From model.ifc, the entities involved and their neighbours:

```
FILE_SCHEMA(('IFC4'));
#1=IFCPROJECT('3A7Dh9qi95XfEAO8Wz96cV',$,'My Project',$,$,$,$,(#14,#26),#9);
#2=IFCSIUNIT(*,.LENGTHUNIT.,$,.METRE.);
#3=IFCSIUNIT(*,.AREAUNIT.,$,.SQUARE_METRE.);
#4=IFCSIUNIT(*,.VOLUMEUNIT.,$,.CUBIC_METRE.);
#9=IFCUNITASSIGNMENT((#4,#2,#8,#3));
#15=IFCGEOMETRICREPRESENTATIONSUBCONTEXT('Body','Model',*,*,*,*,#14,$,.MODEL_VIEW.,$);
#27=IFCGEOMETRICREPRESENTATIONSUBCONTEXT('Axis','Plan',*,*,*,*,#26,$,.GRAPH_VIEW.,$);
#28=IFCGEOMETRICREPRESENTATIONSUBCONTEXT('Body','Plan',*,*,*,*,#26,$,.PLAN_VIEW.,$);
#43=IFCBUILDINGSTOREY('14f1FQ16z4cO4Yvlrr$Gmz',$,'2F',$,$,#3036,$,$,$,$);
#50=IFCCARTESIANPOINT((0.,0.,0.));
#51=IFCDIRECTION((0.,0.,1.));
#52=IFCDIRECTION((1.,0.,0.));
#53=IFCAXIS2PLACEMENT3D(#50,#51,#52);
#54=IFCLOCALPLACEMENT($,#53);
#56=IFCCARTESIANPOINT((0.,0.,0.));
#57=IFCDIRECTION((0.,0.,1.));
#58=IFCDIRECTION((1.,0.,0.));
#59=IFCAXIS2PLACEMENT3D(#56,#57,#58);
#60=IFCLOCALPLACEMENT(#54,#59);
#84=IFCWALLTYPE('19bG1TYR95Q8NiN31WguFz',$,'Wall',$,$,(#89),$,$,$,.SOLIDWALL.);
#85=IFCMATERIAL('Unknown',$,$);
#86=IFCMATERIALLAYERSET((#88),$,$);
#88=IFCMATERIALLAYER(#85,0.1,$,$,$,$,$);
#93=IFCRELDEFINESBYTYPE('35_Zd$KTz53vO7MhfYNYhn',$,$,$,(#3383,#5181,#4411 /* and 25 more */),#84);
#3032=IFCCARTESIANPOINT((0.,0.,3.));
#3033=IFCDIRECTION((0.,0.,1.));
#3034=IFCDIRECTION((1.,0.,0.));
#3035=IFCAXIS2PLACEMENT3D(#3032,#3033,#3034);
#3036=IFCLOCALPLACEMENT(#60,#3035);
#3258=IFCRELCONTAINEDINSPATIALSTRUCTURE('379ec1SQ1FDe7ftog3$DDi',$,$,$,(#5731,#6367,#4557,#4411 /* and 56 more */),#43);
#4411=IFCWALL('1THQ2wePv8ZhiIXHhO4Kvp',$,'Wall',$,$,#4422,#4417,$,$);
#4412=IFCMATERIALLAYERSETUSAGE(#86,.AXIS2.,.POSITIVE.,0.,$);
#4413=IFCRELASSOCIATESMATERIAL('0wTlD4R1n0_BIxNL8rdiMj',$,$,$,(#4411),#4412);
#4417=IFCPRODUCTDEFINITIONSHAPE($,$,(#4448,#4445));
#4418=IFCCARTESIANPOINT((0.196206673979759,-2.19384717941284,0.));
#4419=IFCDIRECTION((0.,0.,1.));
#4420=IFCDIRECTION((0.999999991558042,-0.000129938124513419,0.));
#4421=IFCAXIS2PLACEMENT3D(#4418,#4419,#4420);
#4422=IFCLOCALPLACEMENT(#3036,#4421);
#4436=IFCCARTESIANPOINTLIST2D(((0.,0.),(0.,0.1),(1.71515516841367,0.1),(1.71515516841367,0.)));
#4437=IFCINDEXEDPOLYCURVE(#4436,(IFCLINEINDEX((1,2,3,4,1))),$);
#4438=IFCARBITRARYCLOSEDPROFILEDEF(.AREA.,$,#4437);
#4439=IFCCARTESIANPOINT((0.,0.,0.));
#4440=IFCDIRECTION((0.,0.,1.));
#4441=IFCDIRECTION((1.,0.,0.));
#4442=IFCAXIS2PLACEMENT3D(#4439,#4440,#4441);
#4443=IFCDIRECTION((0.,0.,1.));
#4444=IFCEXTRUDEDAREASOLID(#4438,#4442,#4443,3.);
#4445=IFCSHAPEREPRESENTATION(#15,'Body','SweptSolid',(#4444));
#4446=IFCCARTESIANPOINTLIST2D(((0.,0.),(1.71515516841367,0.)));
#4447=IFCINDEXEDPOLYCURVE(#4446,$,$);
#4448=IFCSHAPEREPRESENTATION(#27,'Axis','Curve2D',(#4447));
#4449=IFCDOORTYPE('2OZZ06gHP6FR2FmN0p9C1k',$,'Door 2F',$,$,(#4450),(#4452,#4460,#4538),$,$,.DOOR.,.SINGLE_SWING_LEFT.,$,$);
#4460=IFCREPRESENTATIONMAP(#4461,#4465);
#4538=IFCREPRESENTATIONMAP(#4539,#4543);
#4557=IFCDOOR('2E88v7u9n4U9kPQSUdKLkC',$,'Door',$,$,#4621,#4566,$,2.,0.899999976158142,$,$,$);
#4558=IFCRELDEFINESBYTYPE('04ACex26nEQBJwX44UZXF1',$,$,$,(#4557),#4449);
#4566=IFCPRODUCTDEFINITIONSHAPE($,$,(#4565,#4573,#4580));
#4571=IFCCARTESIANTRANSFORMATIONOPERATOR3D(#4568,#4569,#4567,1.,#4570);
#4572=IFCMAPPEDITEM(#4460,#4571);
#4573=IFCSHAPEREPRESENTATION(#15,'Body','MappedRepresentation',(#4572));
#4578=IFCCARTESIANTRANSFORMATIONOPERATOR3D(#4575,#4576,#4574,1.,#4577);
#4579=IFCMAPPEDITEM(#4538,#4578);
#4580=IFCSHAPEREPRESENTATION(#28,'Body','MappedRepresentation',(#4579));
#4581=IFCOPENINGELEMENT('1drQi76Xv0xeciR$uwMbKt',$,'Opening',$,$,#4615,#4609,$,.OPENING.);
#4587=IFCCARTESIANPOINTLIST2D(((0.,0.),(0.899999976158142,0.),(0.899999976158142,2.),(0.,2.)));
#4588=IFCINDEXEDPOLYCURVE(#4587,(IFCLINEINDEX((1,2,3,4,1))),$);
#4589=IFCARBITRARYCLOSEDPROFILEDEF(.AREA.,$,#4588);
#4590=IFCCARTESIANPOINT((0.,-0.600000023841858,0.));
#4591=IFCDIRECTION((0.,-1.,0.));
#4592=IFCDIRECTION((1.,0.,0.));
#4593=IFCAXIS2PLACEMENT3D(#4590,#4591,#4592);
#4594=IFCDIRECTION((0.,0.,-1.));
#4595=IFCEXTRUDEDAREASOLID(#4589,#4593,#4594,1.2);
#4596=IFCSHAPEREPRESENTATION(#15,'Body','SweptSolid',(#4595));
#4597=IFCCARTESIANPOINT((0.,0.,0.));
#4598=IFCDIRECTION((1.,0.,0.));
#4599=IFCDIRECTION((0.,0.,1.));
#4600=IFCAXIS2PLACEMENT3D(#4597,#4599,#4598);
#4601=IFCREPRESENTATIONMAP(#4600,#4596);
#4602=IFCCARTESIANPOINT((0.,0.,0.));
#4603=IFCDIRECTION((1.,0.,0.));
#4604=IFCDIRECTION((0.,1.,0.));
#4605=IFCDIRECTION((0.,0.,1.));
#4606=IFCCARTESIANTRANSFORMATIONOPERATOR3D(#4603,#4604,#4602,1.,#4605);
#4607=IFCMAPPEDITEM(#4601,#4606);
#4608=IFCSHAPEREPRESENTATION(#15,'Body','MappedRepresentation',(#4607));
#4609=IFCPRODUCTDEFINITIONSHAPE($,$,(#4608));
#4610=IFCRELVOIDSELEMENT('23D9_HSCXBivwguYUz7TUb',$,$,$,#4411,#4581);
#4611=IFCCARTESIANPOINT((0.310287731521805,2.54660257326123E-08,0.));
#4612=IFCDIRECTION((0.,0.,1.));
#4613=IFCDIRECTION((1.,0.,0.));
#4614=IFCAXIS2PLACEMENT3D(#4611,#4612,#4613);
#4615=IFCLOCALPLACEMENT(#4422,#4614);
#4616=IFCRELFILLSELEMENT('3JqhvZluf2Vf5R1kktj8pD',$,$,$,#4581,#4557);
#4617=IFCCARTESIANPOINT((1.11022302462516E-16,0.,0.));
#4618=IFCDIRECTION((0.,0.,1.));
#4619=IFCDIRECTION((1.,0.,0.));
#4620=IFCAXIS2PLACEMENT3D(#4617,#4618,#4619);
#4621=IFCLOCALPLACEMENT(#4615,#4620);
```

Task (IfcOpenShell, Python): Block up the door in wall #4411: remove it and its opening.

```python
import ifcopenshell
import ifcopenshell.api.feature
import ifcopenshell.api.root
import ifcopenshell.geom
import ifcopenshell.util.shape

model = ifcopenshell.open("model.ifc")
settings = ifcopenshell.geom.settings()


def volume(element):
    """Net volume in cubic metres, openings subtracted."""
    shape = ifcopenshell.geom.create_shape(settings, element)
    return ifcopenshell.util.shape.get_volume(shape.geometry)


door = model.by_guid("2E88v7u9n4U9kPQSUdKLkC")
opening = door.FillsVoids[0].RelatingOpeningElement
wall = opening.VoidsElements[0].RelatingBuildingElement
before = volume(wall)

ifcopenshell.api.root.remove_product(model, product=door)
ifcopenshell.api.feature.remove_feature(model, feature=opening)

after = volume(wall)

print(f"wall volume {before:.3f} -> {after:.3f} m3")

model.write("model_updated.ifc")
```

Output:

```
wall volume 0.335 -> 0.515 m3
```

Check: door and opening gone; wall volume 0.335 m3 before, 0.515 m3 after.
